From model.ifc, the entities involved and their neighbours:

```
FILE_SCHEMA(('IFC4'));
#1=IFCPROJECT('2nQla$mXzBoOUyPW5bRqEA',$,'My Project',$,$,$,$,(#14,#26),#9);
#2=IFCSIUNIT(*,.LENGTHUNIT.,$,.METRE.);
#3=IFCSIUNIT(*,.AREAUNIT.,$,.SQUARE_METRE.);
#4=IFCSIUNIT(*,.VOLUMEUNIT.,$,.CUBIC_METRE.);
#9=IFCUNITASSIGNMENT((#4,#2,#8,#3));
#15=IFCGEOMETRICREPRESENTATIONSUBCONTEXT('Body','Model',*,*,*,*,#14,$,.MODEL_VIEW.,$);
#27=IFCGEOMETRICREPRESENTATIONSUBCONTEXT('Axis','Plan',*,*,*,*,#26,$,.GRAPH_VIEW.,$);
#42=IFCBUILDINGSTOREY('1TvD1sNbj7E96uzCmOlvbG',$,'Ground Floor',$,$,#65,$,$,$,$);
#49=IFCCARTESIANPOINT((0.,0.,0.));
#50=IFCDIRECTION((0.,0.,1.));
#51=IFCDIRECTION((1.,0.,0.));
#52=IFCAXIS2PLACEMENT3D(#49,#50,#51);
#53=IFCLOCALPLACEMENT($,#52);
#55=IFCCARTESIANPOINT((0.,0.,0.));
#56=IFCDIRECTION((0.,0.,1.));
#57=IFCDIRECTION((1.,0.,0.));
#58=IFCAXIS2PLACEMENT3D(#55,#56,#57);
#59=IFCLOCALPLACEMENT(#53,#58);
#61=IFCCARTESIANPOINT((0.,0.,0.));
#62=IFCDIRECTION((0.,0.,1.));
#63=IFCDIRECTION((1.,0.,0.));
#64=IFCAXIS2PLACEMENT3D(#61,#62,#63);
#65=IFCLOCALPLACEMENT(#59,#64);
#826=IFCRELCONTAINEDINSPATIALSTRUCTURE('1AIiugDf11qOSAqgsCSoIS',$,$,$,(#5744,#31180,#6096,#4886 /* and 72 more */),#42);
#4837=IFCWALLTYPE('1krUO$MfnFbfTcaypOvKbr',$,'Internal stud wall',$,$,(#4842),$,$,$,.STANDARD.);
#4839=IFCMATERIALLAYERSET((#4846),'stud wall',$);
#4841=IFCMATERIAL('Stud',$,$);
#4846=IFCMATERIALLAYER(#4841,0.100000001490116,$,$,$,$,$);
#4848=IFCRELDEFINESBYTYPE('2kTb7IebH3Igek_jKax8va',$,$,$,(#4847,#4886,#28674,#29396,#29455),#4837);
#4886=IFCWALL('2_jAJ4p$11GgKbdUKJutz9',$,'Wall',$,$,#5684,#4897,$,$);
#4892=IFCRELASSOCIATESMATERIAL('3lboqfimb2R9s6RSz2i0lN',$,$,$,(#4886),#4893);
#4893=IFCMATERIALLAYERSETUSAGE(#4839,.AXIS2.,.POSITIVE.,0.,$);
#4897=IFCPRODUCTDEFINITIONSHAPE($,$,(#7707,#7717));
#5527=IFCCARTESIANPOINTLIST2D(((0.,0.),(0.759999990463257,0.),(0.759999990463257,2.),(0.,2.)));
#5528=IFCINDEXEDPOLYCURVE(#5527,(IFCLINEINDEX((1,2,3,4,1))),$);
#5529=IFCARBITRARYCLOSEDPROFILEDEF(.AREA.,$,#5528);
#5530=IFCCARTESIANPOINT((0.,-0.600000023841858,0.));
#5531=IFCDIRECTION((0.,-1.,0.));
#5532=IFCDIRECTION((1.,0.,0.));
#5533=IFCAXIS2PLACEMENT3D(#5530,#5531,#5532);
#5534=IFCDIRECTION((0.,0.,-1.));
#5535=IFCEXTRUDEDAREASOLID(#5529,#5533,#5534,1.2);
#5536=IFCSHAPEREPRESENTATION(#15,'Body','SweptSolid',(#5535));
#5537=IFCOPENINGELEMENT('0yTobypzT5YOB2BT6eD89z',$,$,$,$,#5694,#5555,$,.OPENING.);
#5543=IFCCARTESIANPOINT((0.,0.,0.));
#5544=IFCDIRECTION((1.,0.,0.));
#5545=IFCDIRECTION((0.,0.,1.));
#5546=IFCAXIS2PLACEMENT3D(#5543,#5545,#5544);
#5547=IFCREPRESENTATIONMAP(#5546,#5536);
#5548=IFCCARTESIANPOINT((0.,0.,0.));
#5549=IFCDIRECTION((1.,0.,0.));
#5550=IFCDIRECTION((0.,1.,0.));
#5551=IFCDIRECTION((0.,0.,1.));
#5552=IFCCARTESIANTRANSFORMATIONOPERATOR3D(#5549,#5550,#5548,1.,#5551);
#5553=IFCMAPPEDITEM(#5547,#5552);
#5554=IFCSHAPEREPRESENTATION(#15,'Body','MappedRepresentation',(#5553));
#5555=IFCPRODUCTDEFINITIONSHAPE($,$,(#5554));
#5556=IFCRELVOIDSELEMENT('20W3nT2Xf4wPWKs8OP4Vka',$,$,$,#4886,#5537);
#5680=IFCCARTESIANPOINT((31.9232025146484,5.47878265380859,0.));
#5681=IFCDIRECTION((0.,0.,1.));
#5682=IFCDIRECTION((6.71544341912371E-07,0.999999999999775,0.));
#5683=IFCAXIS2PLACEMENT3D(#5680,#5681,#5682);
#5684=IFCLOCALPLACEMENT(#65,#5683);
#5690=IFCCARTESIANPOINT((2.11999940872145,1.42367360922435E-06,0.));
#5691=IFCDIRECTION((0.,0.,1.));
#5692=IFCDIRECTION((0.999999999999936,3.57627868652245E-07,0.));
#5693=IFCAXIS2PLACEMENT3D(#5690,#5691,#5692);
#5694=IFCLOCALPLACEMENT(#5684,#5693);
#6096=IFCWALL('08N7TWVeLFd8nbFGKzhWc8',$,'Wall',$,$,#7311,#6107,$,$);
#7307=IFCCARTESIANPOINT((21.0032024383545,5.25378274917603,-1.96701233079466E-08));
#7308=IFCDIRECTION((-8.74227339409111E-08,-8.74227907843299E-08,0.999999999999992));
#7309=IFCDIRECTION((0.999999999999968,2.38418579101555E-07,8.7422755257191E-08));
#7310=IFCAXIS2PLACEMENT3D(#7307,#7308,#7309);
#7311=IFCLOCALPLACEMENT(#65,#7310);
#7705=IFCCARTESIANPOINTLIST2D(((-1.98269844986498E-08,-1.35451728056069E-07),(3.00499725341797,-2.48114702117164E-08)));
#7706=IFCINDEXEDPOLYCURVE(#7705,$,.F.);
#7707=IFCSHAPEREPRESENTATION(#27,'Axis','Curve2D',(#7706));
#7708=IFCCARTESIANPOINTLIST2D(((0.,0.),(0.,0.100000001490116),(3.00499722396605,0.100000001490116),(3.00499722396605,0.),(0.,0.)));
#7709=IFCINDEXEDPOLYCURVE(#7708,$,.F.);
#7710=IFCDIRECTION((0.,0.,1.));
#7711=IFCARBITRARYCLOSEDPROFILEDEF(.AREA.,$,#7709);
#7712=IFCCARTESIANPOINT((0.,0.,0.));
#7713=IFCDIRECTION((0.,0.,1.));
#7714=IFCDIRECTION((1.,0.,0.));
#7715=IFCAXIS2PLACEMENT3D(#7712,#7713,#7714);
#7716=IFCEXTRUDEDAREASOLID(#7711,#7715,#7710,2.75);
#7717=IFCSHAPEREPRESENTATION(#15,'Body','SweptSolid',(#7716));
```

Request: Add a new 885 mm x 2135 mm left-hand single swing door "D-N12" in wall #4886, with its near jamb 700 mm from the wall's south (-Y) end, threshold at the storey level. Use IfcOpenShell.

```python
import numpy as np
import ifcopenshell
import ifcopenshell.api.feature
import ifcopenshell.api.geometry
import ifcopenshell.api.root
import ifcopenshell.api.spatial
import ifcopenshell.geom
import ifcopenshell.util.element
import ifcopenshell.util.placement
import ifcopenshell.util.representation
import ifcopenshell.util.shape
import ifcopenshell.util.unit

model = ifcopenshell.open("model.ifc")
unit_scale = ifcopenshell.util.unit.calculate_unit_scale(model)
settings = ifcopenshell.geom.settings()


def volume(element):
    """Net volume in cubic metres, openings subtracted."""
    shape = ifcopenshell.geom.create_shape(settings, element)
    return ifcopenshell.util.shape.get_volume(shape.geometry)


wall = model.by_guid("2_jAJ4p$11GgKbdUKJutz9")
storey = ifcopenshell.util.element.get_container(wall, ifc_class="IfcBuildingStorey")
context = ifcopenshell.util.representation.get_context(model, "Model", "Body", "MODEL_VIEW")
before = volume(wall)

width, height, from_end, sill = 0.885, 2.135, 0.7, 0.0  # metres

# The wall runs along its own X axis, and the end named is its -X end.
wall_shape = ifcopenshell.geom.create_shape(settings, wall)
x, y, z = ifcopenshell.util.shape.get_vertices(wall_shape.geometry).T
start = x.min() + from_end
face, thickness = float(y.min()), float(y.max() - y.min())
wall_matrix = ifcopenshell.util.placement.get_local_placement(wall.ObjectPlacement)
level = ifcopenshell.util.placement.get_local_placement(storey.ObjectPlacement)[2, 3]


def in_wall(x, y):
    """Placement at x, y metres in the wall's axes, at sill height."""
    matrix = wall_matrix.copy()
    matrix[:, 3] = wall_matrix @ np.array([x / unit_scale, y / unit_scale, 0.0, 1.0])
    matrix[2, 3] = level + sill / unit_scale
    return matrix


# Opening: a box that overshoots both wall faces by 50 mm.
opening = ifcopenshell.api.root.create_entity(model, ifc_class="IfcOpeningElement", predefined_type="OPENING")
box = ifcopenshell.api.geometry.add_wall_representation(
    model, context=context, length=width, height=height, thickness=thickness + 0.1
)
ifcopenshell.api.geometry.assign_representation(model, product=opening, representation=box)
ifcopenshell.api.geometry.edit_object_placement(model, product=opening, matrix=in_wall(start, face - 0.05), is_si=False)
ifcopenshell.api.feature.add_feature(model, feature=opening, element=wall)

door = ifcopenshell.api.root.create_entity(model, ifc_class="IfcDoor", name="D-N12", predefined_type="DOOR")
door.OverallWidth, door.OverallHeight = width / unit_scale, height / unit_scale
door.OperationType = "SINGLE_SWING_LEFT"
body = ifcopenshell.api.geometry.add_door_representation(
    model,
    context=context,
    overall_width=door.OverallWidth,
    overall_height=door.OverallHeight,
    operation_type="SINGLE_SWING_LEFT",
    lining_properties={"LiningDepth": thickness / unit_scale, "ThresholdDepth": thickness / unit_scale},
)
ifcopenshell.api.geometry.assign_representation(model, product=door, representation=body)
ifcopenshell.api.spatial.assign_container(model, products=[door], relating_structure=storey)
ifcopenshell.api.feature.add_filling(model, opening=opening, element=door)

# The lining spans the wall, so the door starts at the wall face.
ifcopenshell.api.geometry.edit_object_placement(model, product=door, matrix=in_wall(start, face), is_si=False)

after = volume(wall)

print(f"wall volume {before:.3f} -> {after:.3f} m3")

model.write("model-out.ifc")
```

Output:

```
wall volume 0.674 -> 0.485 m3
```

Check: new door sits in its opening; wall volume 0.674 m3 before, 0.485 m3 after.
